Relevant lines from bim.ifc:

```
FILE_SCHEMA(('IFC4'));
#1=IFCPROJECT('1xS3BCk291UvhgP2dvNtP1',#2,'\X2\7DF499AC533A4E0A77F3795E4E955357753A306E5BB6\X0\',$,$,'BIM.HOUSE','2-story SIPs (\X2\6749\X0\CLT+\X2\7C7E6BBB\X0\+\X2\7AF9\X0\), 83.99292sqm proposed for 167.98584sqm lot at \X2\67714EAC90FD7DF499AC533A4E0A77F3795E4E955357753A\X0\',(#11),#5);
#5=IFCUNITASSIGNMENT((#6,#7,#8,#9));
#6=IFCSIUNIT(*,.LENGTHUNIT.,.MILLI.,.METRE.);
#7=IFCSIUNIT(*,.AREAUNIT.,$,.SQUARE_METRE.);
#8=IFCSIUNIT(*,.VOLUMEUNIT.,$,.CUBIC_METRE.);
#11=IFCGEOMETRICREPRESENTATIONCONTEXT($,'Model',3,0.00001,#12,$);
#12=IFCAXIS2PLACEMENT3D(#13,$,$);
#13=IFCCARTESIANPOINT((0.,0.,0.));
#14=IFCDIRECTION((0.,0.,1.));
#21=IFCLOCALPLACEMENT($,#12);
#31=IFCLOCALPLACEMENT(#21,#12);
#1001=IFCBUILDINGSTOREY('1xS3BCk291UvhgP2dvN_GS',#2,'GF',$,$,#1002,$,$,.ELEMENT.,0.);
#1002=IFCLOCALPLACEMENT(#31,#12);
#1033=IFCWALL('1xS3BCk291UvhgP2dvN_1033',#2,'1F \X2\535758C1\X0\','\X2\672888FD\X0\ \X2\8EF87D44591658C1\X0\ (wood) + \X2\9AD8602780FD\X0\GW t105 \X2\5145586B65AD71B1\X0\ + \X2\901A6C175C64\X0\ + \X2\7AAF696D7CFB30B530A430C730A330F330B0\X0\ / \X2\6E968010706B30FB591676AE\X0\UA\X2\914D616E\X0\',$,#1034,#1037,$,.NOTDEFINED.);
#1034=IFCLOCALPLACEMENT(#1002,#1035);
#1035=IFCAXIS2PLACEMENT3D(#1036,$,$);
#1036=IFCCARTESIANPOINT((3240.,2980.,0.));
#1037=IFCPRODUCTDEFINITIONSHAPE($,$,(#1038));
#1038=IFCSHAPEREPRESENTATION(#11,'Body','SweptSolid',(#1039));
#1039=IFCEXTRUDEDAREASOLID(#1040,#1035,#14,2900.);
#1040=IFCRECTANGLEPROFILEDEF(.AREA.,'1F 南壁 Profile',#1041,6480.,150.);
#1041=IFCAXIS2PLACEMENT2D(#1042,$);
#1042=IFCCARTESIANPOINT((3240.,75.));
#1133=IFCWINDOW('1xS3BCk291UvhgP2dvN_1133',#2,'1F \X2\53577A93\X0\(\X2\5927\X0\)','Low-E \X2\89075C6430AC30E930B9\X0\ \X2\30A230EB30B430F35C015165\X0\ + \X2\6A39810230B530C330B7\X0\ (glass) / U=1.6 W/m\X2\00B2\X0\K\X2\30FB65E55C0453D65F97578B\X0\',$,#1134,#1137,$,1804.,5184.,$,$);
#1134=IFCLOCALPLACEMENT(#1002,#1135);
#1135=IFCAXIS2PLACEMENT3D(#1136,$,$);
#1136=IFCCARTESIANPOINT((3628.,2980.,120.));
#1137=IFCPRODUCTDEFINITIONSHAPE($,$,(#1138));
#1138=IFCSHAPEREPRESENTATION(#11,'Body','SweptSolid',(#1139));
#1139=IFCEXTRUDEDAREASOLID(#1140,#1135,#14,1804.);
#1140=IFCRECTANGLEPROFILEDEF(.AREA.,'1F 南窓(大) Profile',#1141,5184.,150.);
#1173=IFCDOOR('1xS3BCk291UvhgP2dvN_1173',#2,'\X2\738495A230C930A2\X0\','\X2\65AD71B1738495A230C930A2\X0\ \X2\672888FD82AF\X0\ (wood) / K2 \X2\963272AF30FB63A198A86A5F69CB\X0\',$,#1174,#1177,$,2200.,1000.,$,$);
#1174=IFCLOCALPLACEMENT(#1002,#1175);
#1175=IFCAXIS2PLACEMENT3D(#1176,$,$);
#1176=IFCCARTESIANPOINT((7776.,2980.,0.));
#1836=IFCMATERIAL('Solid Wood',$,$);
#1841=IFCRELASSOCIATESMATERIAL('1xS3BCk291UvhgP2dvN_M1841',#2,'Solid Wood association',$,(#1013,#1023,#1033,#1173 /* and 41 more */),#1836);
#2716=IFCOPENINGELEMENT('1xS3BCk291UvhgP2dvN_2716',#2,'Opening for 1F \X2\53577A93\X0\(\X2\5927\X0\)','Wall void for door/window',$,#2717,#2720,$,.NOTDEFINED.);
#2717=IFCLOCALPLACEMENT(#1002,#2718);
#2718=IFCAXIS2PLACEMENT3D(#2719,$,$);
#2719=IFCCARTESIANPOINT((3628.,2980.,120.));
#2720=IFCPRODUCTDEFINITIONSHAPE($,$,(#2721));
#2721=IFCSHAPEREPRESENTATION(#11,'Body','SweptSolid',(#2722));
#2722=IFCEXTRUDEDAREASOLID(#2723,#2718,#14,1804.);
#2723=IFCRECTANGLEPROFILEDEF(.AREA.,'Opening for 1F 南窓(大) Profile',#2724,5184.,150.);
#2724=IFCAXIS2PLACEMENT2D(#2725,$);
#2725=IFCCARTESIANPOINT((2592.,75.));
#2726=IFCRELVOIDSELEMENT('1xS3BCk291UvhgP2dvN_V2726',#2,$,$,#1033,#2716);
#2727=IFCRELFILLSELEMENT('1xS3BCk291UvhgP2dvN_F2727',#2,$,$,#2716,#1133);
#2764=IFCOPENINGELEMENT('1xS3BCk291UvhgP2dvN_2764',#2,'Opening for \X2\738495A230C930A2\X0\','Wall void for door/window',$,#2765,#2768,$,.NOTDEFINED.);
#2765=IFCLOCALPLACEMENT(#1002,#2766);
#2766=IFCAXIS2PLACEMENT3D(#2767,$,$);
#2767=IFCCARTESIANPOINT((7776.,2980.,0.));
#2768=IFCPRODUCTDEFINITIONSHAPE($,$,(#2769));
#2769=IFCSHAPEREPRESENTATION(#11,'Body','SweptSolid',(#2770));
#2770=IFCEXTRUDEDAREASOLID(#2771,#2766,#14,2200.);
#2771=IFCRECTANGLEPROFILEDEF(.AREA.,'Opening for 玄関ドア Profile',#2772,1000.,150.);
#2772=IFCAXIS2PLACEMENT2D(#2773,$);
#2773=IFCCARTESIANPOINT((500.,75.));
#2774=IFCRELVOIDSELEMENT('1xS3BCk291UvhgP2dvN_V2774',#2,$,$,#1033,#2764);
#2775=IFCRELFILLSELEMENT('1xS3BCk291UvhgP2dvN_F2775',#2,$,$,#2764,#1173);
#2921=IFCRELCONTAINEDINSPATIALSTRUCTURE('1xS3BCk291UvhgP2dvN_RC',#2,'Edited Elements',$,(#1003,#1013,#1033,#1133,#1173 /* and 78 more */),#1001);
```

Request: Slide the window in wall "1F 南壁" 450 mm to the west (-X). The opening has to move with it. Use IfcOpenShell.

```python
import ifcopenshell
import ifcopenshell.api.geometry
import ifcopenshell.util.placement

model = ifcopenshell.open("bim.ifc")

window = model.by_id(1133)
opening = window.FillsVoids[0].RelatingOpeningElement
wall = opening.VoidsElements[0].RelatingBuildingElement

wall_matrix = ifcopenshell.util.placement.get_local_placement(wall.ObjectPlacement)
shift = wall_matrix[:3, 0] * -450.0
before = ifcopenshell.util.placement.get_local_placement(window.ObjectPlacement)[:3, 3].copy()

# The window is not placed relative to its opening, so move both.
for product in (opening, window):
    matrix = ifcopenshell.util.placement.get_local_placement(product.ObjectPlacement)
    matrix[:3, 3] += shift
    ifcopenshell.api.geometry.edit_object_placement(model, product=product, matrix=matrix, is_si=False)

after = ifcopenshell.util.placement.get_local_placement(window.ObjectPlacement)[:3, 3]
print("window moved by", (after - before).round(3) + 0.0)

model.write("bim_updated.ifc")
```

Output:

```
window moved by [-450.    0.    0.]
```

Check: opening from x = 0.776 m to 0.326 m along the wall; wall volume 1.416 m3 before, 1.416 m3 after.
